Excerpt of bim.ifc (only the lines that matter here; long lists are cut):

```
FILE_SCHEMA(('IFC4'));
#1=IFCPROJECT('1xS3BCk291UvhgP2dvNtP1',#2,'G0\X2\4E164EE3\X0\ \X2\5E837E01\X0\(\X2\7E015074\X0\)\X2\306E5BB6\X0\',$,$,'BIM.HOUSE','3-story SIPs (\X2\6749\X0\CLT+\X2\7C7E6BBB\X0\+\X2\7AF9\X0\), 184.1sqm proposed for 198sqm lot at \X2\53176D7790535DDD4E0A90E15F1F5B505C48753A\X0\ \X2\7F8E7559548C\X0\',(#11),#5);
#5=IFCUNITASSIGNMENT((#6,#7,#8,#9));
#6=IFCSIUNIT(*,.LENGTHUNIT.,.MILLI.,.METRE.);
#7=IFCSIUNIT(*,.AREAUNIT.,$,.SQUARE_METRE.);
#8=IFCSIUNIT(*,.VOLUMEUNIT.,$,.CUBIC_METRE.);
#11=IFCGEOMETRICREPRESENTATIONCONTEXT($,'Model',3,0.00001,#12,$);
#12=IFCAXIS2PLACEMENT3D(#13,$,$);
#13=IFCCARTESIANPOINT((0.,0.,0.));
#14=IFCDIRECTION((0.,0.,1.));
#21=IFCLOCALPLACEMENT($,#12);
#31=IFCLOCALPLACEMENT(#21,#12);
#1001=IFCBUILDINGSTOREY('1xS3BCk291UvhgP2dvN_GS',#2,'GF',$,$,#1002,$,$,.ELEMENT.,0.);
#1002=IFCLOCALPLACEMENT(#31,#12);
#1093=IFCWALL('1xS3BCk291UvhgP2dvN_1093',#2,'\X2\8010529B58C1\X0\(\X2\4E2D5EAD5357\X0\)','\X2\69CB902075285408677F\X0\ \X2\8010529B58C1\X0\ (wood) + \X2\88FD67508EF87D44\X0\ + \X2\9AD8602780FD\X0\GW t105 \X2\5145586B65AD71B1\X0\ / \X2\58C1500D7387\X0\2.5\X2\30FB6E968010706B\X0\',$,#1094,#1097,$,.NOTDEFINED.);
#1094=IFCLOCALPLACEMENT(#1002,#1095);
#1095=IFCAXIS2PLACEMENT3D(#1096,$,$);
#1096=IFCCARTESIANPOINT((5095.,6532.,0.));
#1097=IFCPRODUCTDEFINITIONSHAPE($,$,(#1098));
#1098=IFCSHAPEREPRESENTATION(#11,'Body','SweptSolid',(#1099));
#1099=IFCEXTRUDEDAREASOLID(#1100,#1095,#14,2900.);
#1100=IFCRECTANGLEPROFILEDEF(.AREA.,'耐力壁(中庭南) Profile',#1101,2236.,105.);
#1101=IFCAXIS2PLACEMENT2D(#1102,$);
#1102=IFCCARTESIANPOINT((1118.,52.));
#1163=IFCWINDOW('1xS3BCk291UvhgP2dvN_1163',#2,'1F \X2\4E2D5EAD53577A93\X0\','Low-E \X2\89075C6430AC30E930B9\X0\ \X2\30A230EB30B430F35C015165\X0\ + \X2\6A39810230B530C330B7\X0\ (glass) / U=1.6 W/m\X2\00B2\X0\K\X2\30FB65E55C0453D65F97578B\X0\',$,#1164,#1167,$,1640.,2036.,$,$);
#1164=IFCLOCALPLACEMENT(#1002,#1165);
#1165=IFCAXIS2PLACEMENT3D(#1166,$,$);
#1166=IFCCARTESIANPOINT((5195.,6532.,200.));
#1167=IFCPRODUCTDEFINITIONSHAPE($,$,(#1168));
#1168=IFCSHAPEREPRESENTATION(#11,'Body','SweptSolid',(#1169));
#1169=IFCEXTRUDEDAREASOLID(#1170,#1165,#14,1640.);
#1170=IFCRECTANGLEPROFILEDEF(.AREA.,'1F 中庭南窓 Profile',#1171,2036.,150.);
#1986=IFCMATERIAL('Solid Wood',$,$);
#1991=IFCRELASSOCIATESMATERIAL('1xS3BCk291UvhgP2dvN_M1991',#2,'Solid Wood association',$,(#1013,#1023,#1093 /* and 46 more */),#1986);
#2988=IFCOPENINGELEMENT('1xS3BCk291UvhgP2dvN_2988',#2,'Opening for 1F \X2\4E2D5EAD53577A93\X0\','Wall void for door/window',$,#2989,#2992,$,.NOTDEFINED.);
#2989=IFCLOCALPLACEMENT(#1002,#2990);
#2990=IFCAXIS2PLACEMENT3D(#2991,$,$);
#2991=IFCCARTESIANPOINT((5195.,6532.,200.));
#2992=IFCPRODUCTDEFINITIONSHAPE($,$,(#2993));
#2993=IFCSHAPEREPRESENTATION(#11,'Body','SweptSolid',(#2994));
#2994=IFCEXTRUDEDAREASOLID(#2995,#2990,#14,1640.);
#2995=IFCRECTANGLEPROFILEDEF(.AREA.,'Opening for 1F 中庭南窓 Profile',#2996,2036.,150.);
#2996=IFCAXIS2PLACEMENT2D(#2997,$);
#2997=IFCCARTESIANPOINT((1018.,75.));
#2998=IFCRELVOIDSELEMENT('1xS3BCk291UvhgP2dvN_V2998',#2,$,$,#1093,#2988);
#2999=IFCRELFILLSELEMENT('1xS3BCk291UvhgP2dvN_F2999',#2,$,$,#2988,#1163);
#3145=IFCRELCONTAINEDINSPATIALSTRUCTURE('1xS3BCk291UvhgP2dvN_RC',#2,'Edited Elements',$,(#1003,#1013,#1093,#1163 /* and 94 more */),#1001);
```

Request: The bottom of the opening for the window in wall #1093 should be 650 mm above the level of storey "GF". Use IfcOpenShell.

```python
import numpy as np
import ifcopenshell
import ifcopenshell.api.geometry
import ifcopenshell.geom
import ifcopenshell.util.element
import ifcopenshell.util.placement
import ifcopenshell.util.shape
import ifcopenshell.util.unit

model = ifcopenshell.open("bim.ifc")
unit_scale = ifcopenshell.util.unit.calculate_unit_scale(model)

window = model.by_id(1163)
opening = window.FillsVoids[0].RelatingOpeningElement
storey = ifcopenshell.util.element.get_container(window, ifc_class="IfcBuildingStorey")
level = ifcopenshell.util.placement.get_local_placement(storey.ObjectPlacement)[2, 3]

# The opening's origin need not be at the sill, so measure its lowest point.
shape = ifcopenshell.geom.create_shape(ifcopenshell.geom.settings(), opening)
bottom = ifcopenshell.util.shape.get_shape_bottom_elevation(shape, shape.geometry) / unit_scale
dz = level + 0.65 / unit_scale - bottom

shift = np.array([0.0, 0.0, dz])
# The window is not placed relative to its opening, so move both.
for product in (opening, window):
    matrix = ifcopenshell.util.placement.get_local_placement(product.ObjectPlacement)
    matrix[:3, 3] += shift
    ifcopenshell.api.geometry.edit_object_placement(model, product=product, matrix=matrix, is_si=False)

print(f"moved by {dz * unit_scale:+.3f} m")

model.write("bim_edited.ifc")
```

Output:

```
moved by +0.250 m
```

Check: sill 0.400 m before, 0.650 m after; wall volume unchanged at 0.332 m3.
